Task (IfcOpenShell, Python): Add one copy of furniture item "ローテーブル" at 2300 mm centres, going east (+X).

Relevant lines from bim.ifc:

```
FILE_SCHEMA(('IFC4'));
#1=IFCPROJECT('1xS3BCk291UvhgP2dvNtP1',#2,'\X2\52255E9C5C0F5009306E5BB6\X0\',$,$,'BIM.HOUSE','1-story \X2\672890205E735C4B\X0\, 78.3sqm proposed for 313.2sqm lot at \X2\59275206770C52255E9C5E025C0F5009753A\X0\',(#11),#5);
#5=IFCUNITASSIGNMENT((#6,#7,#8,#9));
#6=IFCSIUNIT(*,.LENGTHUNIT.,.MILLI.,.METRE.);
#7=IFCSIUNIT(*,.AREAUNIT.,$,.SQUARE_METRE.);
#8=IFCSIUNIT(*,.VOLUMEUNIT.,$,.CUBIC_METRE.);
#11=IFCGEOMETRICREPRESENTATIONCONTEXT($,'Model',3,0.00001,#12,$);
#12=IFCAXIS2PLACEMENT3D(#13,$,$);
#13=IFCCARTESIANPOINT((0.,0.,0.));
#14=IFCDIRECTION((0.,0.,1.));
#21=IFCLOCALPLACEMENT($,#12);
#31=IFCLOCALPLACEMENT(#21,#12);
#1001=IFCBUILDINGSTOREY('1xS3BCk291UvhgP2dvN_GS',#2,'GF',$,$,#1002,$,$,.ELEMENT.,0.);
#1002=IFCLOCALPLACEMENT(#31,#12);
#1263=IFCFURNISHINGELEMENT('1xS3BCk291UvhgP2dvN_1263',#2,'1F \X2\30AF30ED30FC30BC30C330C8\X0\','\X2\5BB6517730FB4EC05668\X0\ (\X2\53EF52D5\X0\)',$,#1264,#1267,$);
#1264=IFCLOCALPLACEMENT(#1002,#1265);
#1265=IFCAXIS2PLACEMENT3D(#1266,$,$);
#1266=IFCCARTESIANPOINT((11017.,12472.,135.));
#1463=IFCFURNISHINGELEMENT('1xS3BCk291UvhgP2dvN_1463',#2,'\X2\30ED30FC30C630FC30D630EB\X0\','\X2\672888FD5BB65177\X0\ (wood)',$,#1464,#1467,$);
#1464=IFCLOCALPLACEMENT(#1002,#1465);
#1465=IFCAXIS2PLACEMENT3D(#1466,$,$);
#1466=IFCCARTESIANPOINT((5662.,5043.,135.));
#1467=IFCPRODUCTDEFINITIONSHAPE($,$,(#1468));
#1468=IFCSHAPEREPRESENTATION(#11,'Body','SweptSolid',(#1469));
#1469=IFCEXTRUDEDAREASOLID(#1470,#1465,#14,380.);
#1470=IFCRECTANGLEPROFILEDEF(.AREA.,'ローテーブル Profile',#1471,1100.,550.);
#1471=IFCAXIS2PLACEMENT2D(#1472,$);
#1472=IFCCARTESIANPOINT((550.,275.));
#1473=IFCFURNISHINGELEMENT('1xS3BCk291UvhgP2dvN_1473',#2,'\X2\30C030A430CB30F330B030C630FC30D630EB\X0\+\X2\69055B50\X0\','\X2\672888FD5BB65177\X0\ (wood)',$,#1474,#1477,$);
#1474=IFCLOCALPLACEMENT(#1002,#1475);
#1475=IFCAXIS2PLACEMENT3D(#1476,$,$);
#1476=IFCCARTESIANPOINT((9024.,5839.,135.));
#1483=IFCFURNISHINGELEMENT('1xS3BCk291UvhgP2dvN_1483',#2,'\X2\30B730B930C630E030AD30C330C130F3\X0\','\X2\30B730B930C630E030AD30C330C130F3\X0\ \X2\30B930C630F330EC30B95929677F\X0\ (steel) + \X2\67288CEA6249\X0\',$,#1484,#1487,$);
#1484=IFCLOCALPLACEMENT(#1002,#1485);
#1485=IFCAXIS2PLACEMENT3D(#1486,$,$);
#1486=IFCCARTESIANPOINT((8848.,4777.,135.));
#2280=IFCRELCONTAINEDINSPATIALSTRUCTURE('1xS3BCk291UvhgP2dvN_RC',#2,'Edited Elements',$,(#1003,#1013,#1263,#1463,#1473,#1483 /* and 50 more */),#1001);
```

```python
import numpy as np
import ifcopenshell
import ifcopenshell.api.geometry
import ifcopenshell.api.root
import ifcopenshell.util.element
import ifcopenshell.util.placement

model = ifcopenshell.open("bim.ifc")


def reuse_history(source, copy):
    """copy_class also copies each property set's owner history, people and application; keep the originals."""
    for rel in copy.IsDefinedBy:
        if rel.is_a("IfcRelDefinesByProperties") and (history := rel.RelatingPropertyDefinition.OwnerHistory):
            rel.RelatingPropertyDefinition.OwnerHistory = source.OwnerHistory
            ifcopenshell.util.element.remove_deep2(model, history)


source = model.by_guid("1xS3BCk291UvhgP2dvN_1463")
base = ifcopenshell.util.placement.get_local_placement(source.ObjectPlacement)
step = np.array([1.0, 0.0, 0.0]) * 2300.0

for i in range(1, 2):
    copy = ifcopenshell.api.root.copy_class(model, product=source)
    copy.Representation = ifcopenshell.util.element.copy_deep(
        model, source.Representation, exclude=["IfcGeometricRepresentationContext", "IfcRepresentationMap"]
    )
    reuse_history(source, copy)
    matrix = base.copy()
    matrix[:3, 3] += i * step
    print("added at", matrix[:3, 3].round(3) + 0.0)
    ifcopenshell.api.geometry.edit_object_placement(model, product=copy, matrix=matrix, is_si=False)

model.write("bim_v2.ifc")
```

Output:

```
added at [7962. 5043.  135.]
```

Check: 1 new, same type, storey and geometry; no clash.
